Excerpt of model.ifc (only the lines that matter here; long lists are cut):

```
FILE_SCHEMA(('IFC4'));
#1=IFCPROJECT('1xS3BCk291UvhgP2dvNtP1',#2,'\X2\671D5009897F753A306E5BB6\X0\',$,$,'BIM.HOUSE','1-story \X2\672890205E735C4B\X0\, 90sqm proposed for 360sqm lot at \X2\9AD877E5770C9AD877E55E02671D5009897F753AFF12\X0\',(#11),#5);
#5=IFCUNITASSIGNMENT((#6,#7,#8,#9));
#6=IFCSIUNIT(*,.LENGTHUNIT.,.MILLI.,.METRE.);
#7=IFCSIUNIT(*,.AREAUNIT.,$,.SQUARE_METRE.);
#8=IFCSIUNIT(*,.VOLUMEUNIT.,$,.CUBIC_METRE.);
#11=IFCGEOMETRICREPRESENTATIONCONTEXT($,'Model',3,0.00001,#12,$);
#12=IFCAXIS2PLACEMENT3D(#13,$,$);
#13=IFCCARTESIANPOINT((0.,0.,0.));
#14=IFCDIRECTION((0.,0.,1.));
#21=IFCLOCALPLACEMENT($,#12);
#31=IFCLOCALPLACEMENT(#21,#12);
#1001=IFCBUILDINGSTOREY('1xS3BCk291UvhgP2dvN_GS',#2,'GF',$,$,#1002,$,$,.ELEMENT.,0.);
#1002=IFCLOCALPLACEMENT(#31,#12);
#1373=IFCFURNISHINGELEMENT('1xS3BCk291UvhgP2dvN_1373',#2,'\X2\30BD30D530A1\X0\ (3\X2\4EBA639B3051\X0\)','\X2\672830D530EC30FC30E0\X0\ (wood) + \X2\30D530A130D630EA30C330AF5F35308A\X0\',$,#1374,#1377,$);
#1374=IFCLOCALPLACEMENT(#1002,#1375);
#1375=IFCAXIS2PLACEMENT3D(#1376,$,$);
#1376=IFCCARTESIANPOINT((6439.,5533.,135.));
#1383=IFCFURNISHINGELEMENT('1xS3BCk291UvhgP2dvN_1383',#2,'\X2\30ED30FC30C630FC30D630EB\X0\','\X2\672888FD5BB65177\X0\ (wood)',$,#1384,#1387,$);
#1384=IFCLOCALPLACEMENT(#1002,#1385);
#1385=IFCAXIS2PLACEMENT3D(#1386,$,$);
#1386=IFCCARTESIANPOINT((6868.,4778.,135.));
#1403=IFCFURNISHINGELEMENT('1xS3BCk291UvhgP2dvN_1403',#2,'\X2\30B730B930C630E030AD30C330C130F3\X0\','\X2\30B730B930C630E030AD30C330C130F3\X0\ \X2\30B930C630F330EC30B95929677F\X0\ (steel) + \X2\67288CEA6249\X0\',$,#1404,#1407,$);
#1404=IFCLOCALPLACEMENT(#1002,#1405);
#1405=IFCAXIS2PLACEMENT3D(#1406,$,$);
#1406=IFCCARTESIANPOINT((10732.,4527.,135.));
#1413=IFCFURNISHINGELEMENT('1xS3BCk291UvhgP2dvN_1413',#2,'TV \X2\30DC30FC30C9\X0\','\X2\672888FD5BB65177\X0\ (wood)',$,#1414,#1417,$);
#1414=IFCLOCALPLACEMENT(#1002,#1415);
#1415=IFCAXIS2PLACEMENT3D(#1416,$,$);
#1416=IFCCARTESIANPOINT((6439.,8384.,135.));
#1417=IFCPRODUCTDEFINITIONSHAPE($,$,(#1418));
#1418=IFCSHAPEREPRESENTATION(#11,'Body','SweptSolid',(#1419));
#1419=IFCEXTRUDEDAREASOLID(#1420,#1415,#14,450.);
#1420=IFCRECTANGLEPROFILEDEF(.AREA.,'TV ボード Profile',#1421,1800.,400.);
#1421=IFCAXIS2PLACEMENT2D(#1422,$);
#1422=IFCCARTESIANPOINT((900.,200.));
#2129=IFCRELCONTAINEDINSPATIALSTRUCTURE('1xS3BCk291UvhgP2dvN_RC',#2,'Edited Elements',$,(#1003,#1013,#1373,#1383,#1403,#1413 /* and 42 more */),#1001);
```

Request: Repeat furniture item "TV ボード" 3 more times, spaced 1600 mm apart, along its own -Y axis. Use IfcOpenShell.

```python
import ifcopenshell
import ifcopenshell.api.geometry
import ifcopenshell.api.root
import ifcopenshell.util.element
import ifcopenshell.util.placement

model = ifcopenshell.open("model.ifc")


def reuse_history(source, copy):
    """copy_class also copies each property set's owner history, people and application; keep the originals."""
    for rel in copy.IsDefinedBy:
        if rel.is_a("IfcRelDefinesByProperties") and (history := rel.RelatingPropertyDefinition.OwnerHistory):
            rel.RelatingPropertyDefinition.OwnerHistory = source.OwnerHistory
            ifcopenshell.util.element.remove_deep2(model, history)


source = model.by_guid("1xS3BCk291UvhgP2dvN_1413")
base = ifcopenshell.util.placement.get_local_placement(source.ObjectPlacement)
step = -base[:3, 1] * 1600.0

for i in range(1, 4):
    copy = ifcopenshell.api.root.copy_class(model, product=source)
    copy.Representation = ifcopenshell.util.element.copy_deep(
        model, source.Representation, exclude=["IfcGeometricRepresentationContext", "IfcRepresentationMap"]
    )
    reuse_history(source, copy)
    matrix = base.copy()
    matrix[:3, 3] += i * step
    print("added at", matrix[:3, 3].round(3) + 0.0)
    ifcopenshell.api.geometry.edit_object_placement(model, product=copy, matrix=matrix, is_si=False)

model.write("model_edited.ifc")
```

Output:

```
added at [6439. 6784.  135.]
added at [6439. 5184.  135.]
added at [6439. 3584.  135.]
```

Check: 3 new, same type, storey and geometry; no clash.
